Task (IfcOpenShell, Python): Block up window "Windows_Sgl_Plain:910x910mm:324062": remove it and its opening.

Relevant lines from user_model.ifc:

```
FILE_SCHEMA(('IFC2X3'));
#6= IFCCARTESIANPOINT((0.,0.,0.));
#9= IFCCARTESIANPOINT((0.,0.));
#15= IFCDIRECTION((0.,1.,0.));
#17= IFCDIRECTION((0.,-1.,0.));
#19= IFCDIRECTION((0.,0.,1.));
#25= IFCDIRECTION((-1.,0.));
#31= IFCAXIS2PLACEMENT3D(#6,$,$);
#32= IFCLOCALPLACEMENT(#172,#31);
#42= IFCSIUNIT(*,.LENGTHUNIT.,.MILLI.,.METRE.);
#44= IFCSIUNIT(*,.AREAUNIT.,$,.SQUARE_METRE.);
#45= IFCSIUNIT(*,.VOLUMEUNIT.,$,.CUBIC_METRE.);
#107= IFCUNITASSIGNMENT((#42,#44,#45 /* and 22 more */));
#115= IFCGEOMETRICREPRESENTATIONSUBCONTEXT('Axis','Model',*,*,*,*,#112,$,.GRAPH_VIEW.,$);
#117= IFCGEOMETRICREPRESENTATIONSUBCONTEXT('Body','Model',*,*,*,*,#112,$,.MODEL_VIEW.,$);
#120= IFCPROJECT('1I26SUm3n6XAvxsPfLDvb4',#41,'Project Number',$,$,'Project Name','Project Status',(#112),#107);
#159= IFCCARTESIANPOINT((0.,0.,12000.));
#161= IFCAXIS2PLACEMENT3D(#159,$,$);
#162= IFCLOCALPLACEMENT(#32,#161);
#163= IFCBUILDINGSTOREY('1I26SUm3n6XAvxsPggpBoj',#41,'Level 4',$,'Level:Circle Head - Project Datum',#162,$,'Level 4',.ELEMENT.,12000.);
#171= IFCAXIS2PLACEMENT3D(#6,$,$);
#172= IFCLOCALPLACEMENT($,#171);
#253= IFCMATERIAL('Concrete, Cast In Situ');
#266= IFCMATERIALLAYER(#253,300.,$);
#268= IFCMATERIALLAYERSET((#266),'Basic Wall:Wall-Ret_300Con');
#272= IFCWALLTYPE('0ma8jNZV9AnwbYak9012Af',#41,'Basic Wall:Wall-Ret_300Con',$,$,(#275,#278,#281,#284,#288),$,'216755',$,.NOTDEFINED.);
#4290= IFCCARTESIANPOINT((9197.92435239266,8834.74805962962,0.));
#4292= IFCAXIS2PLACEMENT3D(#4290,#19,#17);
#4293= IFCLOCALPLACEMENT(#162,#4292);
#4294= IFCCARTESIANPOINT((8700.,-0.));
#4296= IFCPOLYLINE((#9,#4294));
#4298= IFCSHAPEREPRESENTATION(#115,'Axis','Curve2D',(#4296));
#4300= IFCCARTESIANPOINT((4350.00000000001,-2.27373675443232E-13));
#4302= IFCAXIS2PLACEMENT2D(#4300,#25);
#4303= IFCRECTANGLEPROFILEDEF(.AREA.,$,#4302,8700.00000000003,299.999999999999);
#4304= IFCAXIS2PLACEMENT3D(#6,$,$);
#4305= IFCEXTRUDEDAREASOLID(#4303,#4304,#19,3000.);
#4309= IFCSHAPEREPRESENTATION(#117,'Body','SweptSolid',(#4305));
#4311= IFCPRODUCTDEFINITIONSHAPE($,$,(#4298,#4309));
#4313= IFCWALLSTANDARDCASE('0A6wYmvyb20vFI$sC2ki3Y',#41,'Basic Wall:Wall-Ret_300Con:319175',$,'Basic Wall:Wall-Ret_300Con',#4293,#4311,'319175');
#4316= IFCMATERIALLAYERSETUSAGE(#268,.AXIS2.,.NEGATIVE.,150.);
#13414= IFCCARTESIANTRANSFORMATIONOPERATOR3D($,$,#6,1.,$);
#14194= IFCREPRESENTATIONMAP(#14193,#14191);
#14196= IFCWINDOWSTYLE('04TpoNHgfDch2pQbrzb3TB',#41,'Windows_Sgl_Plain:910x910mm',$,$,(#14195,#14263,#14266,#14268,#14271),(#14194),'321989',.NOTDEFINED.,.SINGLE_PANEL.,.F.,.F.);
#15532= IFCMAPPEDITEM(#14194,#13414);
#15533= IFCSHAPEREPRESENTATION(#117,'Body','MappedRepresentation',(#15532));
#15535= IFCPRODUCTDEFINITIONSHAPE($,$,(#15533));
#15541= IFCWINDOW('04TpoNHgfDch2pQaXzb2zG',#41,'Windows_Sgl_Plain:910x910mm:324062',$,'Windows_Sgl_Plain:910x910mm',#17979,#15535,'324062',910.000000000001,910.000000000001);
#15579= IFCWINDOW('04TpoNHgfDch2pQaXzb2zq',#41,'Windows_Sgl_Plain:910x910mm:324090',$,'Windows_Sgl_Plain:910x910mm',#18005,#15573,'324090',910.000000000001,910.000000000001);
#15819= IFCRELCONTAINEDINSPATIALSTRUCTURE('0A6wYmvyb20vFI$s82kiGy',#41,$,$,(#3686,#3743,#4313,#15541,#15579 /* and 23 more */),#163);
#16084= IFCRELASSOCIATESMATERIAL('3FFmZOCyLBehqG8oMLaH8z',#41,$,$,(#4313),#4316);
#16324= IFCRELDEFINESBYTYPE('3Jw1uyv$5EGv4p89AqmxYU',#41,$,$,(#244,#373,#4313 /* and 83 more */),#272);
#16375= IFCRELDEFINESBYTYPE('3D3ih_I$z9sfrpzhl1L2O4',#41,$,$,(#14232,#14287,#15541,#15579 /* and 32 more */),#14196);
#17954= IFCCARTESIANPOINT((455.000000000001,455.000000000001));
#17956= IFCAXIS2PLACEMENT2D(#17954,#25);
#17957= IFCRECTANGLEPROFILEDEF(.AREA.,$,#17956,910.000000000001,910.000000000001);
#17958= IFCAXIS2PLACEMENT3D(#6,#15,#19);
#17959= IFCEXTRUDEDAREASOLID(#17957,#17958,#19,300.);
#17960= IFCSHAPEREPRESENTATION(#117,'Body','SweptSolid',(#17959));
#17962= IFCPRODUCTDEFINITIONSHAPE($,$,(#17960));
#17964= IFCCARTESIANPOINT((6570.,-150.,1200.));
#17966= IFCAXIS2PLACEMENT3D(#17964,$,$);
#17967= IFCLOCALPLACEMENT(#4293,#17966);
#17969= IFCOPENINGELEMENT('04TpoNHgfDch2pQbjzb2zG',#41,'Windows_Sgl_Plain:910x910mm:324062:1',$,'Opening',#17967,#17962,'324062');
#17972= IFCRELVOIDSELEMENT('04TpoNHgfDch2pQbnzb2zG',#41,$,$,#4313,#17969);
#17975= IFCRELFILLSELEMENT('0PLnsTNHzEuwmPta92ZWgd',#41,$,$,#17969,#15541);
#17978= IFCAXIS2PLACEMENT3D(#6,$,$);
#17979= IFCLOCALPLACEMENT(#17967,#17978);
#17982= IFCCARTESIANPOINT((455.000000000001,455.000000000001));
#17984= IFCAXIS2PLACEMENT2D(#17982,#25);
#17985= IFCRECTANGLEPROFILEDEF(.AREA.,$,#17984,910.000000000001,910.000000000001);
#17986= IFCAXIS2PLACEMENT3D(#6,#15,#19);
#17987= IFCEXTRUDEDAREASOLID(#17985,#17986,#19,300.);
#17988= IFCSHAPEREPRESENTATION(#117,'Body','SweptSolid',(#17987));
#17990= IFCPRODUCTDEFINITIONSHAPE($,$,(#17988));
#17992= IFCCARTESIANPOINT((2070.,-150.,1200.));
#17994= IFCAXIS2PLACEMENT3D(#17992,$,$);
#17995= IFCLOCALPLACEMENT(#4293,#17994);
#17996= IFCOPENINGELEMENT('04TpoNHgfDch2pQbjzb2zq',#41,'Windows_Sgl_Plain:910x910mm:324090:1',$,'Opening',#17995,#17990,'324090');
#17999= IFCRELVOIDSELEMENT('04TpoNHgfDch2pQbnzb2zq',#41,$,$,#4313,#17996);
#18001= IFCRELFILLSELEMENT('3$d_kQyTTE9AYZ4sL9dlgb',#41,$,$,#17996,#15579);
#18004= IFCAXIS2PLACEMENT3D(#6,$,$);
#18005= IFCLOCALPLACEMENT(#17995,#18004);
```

```python
import ifcopenshell
import ifcopenshell.api.feature
import ifcopenshell.api.root
import ifcopenshell.geom
import ifcopenshell.util.shape

model = ifcopenshell.open("user_model.ifc")
settings = ifcopenshell.geom.settings()


def volume(element):
    """Net volume in cubic metres, openings subtracted."""
    shape = ifcopenshell.geom.create_shape(settings, element)
    return ifcopenshell.util.shape.get_volume(shape.geometry)


window = model.by_guid("04TpoNHgfDch2pQaXzb2zG")
opening = window.FillsVoids[0].RelatingOpeningElement
wall = opening.VoidsElements[0].RelatingBuildingElement
before = volume(wall)

ifcopenshell.api.root.remove_product(model, product=window)
ifcopenshell.api.feature.remove_feature(model, feature=opening)

after = volume(wall)

print(f"wall volume {before:.3f} -> {after:.3f} m3")

model.write("user_model-out.ifc")
```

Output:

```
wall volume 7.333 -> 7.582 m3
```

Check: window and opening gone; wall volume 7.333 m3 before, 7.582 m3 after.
